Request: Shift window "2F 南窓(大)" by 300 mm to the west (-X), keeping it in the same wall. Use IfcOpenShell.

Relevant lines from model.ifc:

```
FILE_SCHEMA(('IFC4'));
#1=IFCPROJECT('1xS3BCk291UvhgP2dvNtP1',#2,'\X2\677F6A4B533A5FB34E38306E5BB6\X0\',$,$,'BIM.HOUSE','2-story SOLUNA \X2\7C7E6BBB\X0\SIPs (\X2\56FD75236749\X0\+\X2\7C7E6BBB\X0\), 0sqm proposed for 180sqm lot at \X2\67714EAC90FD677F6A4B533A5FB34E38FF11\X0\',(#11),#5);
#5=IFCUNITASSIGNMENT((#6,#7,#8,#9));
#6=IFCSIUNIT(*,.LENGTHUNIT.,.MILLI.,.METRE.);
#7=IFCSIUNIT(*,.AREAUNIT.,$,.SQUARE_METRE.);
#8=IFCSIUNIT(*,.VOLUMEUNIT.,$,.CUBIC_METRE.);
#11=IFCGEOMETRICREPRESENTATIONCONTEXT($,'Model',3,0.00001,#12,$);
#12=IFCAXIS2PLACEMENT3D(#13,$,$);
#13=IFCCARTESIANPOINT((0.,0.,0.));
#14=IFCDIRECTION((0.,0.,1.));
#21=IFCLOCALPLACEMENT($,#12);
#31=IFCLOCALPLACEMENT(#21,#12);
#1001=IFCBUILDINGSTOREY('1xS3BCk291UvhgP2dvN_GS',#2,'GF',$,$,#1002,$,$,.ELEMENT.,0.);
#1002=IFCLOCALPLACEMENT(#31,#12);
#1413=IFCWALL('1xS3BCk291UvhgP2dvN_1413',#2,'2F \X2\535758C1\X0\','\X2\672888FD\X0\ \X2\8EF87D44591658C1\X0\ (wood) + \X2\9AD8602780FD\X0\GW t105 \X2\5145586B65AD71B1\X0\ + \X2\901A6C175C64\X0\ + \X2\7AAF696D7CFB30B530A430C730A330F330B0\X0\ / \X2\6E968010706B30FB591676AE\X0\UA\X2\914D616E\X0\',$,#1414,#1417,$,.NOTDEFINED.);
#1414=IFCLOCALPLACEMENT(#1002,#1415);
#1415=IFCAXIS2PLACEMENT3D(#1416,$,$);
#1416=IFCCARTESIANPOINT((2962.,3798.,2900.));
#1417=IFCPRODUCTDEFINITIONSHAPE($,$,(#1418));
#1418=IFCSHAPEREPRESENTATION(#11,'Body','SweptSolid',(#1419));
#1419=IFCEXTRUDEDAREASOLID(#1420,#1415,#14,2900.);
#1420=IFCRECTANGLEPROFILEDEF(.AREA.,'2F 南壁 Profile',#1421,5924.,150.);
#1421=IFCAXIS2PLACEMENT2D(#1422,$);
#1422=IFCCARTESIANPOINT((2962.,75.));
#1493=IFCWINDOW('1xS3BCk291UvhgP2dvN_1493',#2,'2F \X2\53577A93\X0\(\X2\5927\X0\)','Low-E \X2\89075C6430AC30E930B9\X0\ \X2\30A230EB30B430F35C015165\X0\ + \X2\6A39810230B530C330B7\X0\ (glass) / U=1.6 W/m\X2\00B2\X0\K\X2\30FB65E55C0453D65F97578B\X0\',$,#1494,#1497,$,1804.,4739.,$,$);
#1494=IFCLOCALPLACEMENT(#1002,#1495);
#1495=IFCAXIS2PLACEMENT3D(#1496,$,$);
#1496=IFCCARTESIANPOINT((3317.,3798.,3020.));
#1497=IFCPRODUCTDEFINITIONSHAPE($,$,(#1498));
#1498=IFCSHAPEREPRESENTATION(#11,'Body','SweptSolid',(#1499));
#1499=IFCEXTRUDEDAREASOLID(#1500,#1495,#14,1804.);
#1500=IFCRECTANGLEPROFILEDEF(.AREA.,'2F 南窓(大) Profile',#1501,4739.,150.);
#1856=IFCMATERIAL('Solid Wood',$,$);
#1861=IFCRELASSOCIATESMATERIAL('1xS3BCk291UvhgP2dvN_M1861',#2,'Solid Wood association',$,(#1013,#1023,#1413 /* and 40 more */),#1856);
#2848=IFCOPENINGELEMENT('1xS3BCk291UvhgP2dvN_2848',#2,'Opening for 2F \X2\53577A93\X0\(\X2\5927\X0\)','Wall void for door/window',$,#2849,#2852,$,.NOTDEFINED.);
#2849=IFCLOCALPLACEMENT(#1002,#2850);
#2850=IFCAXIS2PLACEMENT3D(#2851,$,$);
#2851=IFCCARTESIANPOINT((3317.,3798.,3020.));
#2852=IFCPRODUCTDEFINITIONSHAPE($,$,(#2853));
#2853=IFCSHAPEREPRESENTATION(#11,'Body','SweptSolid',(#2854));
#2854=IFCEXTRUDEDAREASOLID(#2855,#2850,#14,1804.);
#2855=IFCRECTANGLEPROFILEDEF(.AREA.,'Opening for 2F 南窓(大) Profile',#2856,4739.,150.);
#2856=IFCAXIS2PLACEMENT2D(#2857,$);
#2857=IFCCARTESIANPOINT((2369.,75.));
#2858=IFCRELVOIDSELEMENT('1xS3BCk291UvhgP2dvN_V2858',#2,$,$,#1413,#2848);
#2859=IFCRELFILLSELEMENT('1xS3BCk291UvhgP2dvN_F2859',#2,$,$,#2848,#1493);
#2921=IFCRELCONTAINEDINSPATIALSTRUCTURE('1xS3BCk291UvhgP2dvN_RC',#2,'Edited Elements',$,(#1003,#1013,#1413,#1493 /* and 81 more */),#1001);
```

```python
import ifcopenshell
import ifcopenshell.api.geometry
import ifcopenshell.util.placement

model = ifcopenshell.open("model.ifc")

window = model.by_id(1493)
opening = window.FillsVoids[0].RelatingOpeningElement
wall = opening.VoidsElements[0].RelatingBuildingElement

wall_matrix = ifcopenshell.util.placement.get_local_placement(wall.ObjectPlacement)
shift = wall_matrix[:3, 0] * -300.0
before = ifcopenshell.util.placement.get_local_placement(window.ObjectPlacement)[:3, 3].copy()

# The window is not placed relative to its opening, so move both.
for product in (opening, window):
    matrix = ifcopenshell.util.placement.get_local_placement(product.ObjectPlacement)
    matrix[:3, 3] += shift
    ifcopenshell.api.geometry.edit_object_placement(model, product=product, matrix=matrix, is_si=False)

after = ifcopenshell.util.placement.get_local_placement(window.ObjectPlacement)[:3, 3]
print("window moved by", (after - before).round(3) + 0.0)

model.write("model-out.ifc")
```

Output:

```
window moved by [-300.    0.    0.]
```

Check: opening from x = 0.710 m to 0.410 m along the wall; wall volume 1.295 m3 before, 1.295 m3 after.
